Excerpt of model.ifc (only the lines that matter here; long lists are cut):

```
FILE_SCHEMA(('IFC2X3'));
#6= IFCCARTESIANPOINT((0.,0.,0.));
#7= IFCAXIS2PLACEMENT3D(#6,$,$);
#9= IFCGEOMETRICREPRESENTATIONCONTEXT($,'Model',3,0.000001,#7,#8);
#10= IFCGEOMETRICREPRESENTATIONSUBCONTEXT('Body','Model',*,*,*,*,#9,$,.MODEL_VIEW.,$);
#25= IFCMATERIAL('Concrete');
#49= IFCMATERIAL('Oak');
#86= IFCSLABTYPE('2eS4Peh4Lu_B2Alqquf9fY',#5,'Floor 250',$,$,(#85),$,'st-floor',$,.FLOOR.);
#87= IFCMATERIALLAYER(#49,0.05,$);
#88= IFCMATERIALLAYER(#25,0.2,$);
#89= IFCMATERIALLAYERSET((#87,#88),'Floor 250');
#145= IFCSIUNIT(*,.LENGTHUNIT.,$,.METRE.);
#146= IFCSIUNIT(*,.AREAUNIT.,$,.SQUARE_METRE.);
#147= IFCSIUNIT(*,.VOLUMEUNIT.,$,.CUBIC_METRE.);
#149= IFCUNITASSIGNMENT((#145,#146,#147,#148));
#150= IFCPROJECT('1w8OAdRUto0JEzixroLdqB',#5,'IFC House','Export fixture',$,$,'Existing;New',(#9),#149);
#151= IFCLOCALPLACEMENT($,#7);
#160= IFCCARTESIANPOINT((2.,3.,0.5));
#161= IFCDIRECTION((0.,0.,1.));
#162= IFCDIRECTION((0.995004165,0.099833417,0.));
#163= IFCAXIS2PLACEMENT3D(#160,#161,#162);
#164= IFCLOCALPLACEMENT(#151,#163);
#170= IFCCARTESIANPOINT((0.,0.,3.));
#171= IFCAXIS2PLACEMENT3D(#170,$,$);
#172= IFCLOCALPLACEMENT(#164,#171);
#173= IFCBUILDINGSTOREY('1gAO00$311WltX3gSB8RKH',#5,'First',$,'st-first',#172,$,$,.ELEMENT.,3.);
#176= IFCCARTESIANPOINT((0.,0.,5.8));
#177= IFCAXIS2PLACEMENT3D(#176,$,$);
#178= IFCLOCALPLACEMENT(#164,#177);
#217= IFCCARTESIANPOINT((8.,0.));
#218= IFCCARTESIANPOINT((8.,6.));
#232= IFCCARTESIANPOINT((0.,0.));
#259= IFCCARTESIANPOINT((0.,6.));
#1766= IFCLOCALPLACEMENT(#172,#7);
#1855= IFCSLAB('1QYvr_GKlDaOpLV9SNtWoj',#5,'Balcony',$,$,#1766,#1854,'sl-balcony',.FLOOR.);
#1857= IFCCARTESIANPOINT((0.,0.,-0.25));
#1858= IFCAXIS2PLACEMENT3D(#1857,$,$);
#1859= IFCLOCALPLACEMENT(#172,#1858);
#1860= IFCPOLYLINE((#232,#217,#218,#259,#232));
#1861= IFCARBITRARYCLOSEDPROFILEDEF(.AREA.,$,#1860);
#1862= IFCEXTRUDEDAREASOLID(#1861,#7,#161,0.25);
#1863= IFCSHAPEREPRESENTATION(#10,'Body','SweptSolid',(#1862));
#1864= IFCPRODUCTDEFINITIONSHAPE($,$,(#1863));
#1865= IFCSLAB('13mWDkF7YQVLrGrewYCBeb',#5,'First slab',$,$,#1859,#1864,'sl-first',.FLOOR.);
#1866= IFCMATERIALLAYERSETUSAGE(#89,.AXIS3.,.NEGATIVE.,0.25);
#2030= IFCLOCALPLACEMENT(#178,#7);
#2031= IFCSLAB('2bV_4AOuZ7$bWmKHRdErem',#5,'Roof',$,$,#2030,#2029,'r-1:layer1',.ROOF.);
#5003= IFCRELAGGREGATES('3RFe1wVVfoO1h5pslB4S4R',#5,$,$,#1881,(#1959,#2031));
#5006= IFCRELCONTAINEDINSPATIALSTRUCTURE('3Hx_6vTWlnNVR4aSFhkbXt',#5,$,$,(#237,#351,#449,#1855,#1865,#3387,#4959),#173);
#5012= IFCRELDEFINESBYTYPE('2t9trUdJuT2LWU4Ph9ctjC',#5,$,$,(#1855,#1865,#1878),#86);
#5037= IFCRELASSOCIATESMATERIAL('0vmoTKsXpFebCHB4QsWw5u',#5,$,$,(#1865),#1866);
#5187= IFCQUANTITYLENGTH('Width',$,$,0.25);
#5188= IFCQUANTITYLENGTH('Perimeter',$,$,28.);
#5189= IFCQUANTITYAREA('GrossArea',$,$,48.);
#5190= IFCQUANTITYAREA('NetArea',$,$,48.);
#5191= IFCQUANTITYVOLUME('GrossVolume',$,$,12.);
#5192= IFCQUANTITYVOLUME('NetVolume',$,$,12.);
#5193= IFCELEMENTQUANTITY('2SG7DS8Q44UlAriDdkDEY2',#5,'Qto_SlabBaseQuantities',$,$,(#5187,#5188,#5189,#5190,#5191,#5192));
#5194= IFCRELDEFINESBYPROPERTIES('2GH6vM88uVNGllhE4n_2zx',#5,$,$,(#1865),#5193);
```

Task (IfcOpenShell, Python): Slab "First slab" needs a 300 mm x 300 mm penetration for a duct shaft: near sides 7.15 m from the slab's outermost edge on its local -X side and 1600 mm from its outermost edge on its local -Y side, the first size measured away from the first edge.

```python
import numpy as np
import ifcopenshell
import ifcopenshell.api.feature
import ifcopenshell.api.geometry
import ifcopenshell.api.pset
import ifcopenshell.api.root
import ifcopenshell.geom
import ifcopenshell.util.element
import ifcopenshell.util.placement
import ifcopenshell.util.representation
import ifcopenshell.util.shape
import ifcopenshell.util.unit

model = ifcopenshell.open("model.ifc")
unit_scale = ifcopenshell.util.unit.calculate_unit_scale(model)
area_scale = ifcopenshell.util.unit.calculate_unit_scale(model, "AREAUNIT")
volume_scale = ifcopenshell.util.unit.calculate_unit_scale(model, "VOLUMEUNIT")
settings = ifcopenshell.geom.settings()


def volume(element):
    """Net volume in cubic metres, openings subtracted."""
    shape = ifcopenshell.geom.create_shape(settings, element)
    return ifcopenshell.util.shape.get_volume(shape.geometry)


slab = model.by_guid("13mWDkF7YQVLrGrewYCBeb")
before = volume(slab)

# Extent in the slab's own axes, in metres. The edges named are its -X and -Y sides.
slab_shape = ifcopenshell.geom.create_shape(settings, slab)
vertices = ifcopenshell.util.shape.get_vertices(slab_shape.geometry)
x_min, y_min, bottom = vertices.min(axis=0)
top = vertices[:, 2].max()

opening = ifcopenshell.api.root.create_entity(model, ifc_class="IfcOpeningElement", name="Duct shaft opening")
context = ifcopenshell.util.representation.get_context(model, "Model", "Body", "MODEL_VIEW")
width, depth = 0.3, 0.3
outline = [(0.0, 0.0), (width, 0.0), (width, depth), (0.0, depth), (0.0, 0.0)]
# Overshoot both faces by 50 mm so the cut is clean.
shape = ifcopenshell.api.geometry.add_slab_representation(
    model, context=context, depth=top - bottom + 0.1, polyline=outline
)
ifcopenshell.api.geometry.assign_representation(model, product=opening, representation=shape)

matrix = ifcopenshell.util.placement.get_local_placement(slab.ObjectPlacement)
matrix[:, 3] = matrix @ np.append(np.array([x_min + 7.15, y_min + 1.6, bottom - 0.05]) / unit_scale, 1.0)
ifcopenshell.api.geometry.edit_object_placement(model, product=opening, matrix=matrix, is_si=False)
ifcopenshell.api.feature.add_feature(model, feature=opening, element=slab)

after = volume(slab)

# Update the slab's stored quantities.
qto = model.by_id(ifcopenshell.util.element.get_pset(slab, "Qto_SlabBaseQuantities", should_inherit=False)["id"])
ifcopenshell.api.pset.edit_qto(model, qto=qto, properties={
    "NetArea": after / (top - bottom) / area_scale,
    "NetVolume": after / volume_scale,
})

print(f"slab volume {before:.3f} -> {after:.3f} m3")

model.write("model-out.ifc")
```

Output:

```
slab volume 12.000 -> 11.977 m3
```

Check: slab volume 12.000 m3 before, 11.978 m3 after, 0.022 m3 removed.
